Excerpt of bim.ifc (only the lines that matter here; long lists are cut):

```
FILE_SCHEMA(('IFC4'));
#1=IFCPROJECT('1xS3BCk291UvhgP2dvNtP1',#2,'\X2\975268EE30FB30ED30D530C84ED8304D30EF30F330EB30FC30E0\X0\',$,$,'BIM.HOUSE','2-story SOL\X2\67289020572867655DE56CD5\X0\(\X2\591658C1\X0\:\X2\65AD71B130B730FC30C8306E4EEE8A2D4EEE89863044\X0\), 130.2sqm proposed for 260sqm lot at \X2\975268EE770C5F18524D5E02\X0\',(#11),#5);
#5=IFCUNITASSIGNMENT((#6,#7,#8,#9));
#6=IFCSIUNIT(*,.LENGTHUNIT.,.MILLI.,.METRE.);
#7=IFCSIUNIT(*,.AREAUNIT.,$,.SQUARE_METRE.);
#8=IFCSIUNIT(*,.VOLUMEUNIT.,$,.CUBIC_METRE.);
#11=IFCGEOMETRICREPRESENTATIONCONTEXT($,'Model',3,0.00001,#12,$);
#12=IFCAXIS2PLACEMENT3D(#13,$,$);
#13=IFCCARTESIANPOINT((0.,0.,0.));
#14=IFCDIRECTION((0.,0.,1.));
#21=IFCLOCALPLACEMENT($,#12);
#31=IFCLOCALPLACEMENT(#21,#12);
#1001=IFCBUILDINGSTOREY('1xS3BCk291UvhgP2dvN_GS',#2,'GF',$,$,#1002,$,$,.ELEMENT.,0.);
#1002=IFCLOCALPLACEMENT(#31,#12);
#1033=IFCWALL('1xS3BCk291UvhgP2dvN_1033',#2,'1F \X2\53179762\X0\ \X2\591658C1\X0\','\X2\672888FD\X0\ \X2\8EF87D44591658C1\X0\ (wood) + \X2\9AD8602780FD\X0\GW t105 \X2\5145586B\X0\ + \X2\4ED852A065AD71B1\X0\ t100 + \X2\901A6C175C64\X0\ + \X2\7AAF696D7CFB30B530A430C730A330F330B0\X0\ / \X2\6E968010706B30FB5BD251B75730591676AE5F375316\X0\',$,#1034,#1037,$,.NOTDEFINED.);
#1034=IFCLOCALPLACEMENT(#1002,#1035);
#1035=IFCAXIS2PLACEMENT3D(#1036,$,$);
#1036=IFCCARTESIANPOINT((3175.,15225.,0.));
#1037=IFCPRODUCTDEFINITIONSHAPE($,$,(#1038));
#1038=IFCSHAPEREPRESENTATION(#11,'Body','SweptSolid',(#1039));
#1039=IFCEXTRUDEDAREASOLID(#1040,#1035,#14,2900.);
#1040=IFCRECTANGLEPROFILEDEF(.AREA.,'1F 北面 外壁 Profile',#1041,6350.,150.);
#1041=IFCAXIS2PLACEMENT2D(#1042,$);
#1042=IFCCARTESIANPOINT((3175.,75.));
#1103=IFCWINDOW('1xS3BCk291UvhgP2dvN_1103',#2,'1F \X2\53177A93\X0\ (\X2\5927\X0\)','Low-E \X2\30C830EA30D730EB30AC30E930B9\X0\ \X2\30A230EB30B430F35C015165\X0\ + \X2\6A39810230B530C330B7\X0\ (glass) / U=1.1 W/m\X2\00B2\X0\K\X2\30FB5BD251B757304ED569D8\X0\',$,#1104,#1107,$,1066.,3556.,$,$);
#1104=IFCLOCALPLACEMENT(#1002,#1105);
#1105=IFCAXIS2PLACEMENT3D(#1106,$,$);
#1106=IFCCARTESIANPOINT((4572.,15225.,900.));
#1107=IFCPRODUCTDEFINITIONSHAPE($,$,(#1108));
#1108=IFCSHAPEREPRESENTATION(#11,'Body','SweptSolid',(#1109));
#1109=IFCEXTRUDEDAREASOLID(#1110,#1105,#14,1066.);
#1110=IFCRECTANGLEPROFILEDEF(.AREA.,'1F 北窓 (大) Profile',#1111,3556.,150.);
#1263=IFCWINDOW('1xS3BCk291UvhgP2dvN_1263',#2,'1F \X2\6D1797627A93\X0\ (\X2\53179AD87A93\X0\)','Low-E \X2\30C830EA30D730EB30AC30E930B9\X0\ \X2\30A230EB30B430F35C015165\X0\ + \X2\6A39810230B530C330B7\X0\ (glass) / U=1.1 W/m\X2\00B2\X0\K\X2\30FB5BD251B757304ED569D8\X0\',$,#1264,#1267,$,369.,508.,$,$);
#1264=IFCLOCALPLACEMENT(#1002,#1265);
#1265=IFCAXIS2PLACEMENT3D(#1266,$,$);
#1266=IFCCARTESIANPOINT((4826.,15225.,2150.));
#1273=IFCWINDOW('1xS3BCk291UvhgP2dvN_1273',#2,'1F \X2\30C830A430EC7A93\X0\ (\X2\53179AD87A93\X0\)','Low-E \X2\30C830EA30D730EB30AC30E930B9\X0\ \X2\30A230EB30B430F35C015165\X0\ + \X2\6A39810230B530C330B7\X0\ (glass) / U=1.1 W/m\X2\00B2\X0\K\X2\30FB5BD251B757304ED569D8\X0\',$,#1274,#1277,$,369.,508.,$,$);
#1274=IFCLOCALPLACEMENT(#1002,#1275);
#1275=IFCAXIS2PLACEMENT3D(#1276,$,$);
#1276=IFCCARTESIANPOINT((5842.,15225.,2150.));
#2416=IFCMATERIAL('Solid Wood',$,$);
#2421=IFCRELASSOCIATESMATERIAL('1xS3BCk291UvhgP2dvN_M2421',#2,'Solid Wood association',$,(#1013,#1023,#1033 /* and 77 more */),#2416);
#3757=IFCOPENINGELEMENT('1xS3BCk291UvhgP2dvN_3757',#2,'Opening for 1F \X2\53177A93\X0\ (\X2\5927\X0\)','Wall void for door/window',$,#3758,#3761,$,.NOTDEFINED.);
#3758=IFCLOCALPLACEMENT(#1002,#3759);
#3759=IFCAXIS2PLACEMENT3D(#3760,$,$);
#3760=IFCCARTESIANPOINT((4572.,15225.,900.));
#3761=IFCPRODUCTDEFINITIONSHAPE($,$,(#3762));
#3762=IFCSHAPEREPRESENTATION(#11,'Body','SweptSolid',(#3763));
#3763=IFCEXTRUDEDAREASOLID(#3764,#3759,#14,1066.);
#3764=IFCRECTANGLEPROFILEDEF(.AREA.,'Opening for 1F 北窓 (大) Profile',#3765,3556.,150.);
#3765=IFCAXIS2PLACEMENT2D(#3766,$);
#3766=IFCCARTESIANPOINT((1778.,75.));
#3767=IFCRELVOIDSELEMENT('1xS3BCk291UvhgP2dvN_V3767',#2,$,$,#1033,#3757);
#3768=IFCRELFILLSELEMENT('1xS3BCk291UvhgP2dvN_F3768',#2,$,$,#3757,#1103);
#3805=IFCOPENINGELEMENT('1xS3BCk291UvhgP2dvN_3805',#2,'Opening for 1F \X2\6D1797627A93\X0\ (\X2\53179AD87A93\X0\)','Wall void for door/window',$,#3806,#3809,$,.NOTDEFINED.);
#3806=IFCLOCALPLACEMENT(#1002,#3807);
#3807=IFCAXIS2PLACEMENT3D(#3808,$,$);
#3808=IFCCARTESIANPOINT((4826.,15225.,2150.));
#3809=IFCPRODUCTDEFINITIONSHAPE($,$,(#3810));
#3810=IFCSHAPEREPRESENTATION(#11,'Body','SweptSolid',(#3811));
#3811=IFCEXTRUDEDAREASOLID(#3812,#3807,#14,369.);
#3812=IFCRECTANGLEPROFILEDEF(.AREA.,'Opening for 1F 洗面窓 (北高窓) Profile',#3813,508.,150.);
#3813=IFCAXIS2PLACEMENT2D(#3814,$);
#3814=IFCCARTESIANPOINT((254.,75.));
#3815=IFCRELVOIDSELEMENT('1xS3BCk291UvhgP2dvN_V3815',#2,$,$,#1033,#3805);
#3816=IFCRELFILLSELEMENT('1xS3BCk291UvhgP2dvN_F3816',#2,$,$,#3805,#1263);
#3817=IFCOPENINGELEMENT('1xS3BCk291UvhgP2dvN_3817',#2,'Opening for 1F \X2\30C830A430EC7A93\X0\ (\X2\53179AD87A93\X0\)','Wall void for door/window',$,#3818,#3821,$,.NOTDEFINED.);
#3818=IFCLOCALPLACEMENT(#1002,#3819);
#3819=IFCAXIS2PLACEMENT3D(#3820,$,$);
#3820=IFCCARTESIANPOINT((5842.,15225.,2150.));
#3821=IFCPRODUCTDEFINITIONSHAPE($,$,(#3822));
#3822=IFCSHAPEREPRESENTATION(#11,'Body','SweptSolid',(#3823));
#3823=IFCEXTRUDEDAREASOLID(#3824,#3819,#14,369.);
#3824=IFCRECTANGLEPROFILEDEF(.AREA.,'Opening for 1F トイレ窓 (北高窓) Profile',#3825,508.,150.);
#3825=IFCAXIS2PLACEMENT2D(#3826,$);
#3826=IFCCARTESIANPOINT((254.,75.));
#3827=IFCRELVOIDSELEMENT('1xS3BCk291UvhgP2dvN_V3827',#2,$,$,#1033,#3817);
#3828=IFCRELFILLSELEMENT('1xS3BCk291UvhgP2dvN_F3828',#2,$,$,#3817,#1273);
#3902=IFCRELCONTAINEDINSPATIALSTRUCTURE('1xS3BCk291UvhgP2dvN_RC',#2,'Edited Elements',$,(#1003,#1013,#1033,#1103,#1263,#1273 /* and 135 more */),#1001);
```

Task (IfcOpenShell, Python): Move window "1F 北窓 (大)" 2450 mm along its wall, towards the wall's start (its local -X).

```python
import ifcopenshell
import ifcopenshell.api.geometry
import ifcopenshell.util.placement
import ifcopenshell.util.unit

model = ifcopenshell.open("bim.ifc")
unit_scale = ifcopenshell.util.unit.calculate_unit_scale(model)

window = model.by_guid("1xS3BCk291UvhgP2dvN_1103")
opening = window.FillsVoids[0].RelatingOpeningElement
wall = opening.VoidsElements[0].RelatingBuildingElement

wall_matrix = ifcopenshell.util.placement.get_local_placement(wall.ObjectPlacement)
shift = wall_matrix[:3, 0] * -2.45 / unit_scale
before = ifcopenshell.util.placement.get_local_placement(window.ObjectPlacement)[:3, 3].copy()

# The window is not placed relative to its opening, so move both.
for product in (opening, window):
    matrix = ifcopenshell.util.placement.get_local_placement(product.ObjectPlacement)
    matrix[:3, 3] += shift
    ifcopenshell.api.geometry.edit_object_placement(model, product=product, matrix=matrix, is_si=False)

after = ifcopenshell.util.placement.get_local_placement(window.ObjectPlacement)[:3, 3]
print("window moved by", (after - before).round(3) + 0.0)

model.write("bim_updated.ifc")
```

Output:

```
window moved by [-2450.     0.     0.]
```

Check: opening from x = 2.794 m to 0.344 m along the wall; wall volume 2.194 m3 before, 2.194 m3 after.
